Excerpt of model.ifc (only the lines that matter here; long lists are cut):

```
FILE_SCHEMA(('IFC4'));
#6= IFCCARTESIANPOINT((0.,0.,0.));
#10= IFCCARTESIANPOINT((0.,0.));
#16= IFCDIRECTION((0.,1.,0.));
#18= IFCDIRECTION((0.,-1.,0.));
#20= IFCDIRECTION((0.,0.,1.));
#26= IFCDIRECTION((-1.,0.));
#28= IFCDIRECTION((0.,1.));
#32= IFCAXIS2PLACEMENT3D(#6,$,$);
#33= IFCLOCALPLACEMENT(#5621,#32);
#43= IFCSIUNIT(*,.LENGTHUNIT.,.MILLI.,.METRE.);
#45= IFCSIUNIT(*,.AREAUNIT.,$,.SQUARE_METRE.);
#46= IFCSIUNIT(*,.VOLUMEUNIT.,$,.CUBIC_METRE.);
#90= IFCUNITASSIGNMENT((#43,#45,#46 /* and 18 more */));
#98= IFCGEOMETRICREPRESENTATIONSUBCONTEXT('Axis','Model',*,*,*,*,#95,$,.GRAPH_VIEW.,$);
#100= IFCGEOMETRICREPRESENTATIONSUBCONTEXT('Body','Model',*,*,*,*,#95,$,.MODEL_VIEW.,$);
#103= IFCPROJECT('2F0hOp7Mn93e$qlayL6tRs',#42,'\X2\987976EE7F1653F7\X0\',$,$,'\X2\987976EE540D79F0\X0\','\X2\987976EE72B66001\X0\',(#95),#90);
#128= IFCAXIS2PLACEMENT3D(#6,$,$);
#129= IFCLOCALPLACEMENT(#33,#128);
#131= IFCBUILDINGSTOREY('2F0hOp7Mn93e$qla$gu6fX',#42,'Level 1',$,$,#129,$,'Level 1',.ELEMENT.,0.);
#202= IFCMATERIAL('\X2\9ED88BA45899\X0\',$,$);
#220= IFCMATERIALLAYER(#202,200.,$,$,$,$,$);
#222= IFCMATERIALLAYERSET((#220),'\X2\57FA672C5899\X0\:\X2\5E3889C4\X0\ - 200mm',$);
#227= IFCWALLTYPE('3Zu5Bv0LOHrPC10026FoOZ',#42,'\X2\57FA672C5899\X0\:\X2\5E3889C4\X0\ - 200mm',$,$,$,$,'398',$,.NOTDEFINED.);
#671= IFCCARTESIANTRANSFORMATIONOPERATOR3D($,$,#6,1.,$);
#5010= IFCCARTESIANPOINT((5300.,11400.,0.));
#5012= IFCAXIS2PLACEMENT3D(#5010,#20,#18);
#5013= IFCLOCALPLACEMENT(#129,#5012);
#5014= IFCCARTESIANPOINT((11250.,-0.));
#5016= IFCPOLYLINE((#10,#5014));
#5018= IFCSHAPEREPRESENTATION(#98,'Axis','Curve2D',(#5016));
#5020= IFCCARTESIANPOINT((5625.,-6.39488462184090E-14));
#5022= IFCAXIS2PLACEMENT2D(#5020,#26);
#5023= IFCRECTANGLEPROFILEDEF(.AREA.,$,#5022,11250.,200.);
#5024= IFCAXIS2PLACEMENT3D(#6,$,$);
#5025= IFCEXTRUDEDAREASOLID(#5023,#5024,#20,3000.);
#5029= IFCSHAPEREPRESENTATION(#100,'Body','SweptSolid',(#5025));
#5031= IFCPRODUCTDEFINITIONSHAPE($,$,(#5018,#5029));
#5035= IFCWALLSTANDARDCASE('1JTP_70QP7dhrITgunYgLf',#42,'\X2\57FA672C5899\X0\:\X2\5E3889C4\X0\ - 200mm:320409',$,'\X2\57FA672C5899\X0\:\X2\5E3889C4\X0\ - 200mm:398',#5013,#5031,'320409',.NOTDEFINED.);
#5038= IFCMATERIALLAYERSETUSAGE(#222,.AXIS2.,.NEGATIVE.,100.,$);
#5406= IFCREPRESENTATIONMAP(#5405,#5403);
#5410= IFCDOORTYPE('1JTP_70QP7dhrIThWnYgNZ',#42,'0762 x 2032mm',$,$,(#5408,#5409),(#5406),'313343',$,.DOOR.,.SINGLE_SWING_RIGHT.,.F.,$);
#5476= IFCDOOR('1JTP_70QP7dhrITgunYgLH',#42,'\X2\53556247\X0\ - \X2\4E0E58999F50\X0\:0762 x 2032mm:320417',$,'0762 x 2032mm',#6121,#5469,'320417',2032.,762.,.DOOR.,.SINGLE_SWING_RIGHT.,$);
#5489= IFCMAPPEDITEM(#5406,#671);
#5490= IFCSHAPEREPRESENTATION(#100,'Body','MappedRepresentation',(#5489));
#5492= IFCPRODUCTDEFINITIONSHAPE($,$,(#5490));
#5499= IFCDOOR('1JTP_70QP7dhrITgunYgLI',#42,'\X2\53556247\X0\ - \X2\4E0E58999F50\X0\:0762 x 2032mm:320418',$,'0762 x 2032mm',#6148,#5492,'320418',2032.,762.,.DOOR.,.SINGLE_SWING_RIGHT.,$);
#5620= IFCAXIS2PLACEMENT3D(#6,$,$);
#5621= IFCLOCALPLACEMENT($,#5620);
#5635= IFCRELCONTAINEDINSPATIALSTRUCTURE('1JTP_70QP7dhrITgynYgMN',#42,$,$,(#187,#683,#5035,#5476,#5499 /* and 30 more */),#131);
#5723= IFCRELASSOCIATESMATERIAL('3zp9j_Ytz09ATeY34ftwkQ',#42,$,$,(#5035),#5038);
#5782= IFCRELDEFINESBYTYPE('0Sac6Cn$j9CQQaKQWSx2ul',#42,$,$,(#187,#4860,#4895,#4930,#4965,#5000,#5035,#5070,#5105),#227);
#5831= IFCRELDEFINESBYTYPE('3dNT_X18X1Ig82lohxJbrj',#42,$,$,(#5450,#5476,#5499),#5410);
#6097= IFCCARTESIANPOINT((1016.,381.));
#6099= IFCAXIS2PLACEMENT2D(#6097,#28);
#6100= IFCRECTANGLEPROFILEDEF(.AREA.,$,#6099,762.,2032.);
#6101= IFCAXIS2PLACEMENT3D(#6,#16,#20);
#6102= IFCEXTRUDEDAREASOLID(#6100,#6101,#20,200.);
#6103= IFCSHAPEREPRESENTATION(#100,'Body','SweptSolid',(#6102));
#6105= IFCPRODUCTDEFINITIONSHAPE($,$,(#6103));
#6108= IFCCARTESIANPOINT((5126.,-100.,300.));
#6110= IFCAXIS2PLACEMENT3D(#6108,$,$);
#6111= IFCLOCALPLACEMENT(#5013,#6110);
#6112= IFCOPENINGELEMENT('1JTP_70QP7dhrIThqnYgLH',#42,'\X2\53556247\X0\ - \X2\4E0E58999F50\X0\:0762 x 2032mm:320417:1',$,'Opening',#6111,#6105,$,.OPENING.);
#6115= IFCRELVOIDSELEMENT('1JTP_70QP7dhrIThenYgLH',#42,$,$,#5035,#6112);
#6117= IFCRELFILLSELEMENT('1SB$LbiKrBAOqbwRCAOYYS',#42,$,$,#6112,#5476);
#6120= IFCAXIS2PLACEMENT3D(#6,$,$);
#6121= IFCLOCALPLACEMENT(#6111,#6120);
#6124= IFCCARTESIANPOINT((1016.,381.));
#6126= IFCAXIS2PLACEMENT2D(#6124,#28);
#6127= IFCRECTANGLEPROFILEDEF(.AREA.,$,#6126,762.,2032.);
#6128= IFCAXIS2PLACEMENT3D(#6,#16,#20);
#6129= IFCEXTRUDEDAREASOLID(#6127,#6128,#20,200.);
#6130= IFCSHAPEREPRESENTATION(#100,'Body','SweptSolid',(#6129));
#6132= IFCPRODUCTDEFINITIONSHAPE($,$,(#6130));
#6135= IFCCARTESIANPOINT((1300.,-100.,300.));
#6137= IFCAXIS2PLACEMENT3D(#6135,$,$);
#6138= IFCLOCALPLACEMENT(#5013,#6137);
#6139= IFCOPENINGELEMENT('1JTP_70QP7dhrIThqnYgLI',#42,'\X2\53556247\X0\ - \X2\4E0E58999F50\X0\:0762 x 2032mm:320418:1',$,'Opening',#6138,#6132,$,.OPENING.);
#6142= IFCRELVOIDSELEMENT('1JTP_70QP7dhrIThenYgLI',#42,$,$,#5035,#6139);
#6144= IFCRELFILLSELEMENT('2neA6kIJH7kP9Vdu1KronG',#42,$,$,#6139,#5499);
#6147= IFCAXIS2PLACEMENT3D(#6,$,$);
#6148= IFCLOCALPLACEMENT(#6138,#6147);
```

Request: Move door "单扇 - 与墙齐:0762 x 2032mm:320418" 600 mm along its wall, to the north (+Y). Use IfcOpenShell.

```python
import ifcopenshell
import ifcopenshell.api.geometry
import ifcopenshell.util.placement

model = ifcopenshell.open("model.ifc")

door = model.by_id(5499)
opening = door.FillsVoids[0].RelatingOpeningElement
wall = opening.VoidsElements[0].RelatingBuildingElement

wall_matrix = ifcopenshell.util.placement.get_local_placement(wall.ObjectPlacement)
shift = wall_matrix[:3, 0] * -600.0
before = ifcopenshell.util.placement.get_local_placement(door.ObjectPlacement)[:3, 3].copy()

# The door is placed relative to its opening, so it follows when the opening moves.
matrix = ifcopenshell.util.placement.get_local_placement(opening.ObjectPlacement)
matrix[:3, 3] += shift
ifcopenshell.api.geometry.edit_object_placement(
    model, product=opening, matrix=matrix, is_si=False, should_transform_children=True
)

after = ifcopenshell.util.placement.get_local_placement(door.ObjectPlacement)[:3, 3]
print("door moved by", (after - before).round(3) + 0.0)

model.write("model_v2.ifc")
```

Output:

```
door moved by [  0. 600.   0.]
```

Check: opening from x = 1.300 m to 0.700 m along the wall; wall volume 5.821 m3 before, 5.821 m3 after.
